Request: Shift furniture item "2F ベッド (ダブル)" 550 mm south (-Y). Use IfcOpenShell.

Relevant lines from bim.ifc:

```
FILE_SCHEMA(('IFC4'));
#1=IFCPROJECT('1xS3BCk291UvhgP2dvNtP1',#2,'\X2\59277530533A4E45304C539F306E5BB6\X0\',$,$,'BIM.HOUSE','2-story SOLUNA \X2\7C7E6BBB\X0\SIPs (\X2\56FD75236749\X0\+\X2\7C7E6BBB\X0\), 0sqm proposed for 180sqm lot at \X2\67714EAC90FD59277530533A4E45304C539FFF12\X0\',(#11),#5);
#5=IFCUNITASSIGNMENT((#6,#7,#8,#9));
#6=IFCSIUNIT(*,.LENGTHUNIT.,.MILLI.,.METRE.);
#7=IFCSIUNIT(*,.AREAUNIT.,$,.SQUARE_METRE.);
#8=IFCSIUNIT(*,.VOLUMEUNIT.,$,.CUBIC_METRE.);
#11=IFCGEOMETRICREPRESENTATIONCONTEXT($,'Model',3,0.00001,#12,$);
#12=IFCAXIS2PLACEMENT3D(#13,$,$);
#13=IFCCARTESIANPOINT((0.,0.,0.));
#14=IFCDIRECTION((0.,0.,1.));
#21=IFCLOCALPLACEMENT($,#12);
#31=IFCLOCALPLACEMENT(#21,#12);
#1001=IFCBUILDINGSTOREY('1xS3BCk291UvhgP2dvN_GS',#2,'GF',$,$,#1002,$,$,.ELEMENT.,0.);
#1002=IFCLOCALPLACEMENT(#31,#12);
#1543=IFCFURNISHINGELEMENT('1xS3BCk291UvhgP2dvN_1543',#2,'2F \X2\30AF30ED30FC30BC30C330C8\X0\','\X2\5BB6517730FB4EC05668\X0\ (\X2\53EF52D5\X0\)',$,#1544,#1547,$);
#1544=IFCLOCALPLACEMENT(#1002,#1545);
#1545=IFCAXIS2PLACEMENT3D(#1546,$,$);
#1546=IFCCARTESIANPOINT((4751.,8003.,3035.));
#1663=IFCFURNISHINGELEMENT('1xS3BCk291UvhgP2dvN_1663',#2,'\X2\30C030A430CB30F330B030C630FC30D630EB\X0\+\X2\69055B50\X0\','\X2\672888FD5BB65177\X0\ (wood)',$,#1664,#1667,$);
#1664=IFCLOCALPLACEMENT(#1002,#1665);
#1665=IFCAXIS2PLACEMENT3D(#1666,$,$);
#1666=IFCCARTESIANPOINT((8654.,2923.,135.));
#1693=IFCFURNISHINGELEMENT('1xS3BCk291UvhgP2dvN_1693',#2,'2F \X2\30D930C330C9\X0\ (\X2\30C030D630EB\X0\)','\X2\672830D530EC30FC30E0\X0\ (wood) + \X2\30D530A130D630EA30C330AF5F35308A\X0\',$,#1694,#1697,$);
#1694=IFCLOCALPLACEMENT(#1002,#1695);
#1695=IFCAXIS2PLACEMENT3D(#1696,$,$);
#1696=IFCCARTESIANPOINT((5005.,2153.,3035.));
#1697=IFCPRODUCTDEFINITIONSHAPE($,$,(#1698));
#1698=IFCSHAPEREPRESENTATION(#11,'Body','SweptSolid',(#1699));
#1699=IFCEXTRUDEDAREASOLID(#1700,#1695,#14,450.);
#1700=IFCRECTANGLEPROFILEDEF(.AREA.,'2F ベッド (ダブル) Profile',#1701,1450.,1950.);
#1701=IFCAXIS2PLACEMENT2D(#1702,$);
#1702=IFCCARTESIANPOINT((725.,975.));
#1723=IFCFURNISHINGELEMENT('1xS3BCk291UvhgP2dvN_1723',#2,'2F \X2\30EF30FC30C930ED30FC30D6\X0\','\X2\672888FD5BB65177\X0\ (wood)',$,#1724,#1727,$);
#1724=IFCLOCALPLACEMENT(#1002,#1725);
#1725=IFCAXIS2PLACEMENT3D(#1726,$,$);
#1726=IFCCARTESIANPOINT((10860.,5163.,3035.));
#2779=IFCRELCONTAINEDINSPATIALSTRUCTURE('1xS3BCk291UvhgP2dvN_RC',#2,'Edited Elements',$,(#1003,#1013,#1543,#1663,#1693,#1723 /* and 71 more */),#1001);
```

```python
import ifcopenshell
import ifcopenshell.api.geometry
import ifcopenshell.util.placement

model = ifcopenshell.open("bim.ifc")

item = model.by_guid("1xS3BCk291UvhgP2dvN_1693")
matrix = ifcopenshell.util.placement.get_local_placement(item.ObjectPlacement)
matrix[1, 3] -= 550.0
ifcopenshell.api.geometry.edit_object_placement(model, product=item, matrix=matrix, is_si=False)

print(ifcopenshell.util.placement.get_local_placement(item.ObjectPlacement).round(3) + 0.0)

model.write("bim_edited.ifc")
```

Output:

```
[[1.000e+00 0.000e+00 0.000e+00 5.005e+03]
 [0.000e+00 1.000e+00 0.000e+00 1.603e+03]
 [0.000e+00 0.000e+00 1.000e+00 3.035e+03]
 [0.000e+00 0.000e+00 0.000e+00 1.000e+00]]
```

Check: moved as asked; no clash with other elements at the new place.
